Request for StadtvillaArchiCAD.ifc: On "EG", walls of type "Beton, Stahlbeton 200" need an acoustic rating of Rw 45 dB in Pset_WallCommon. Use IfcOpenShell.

First a look at what the model holds.

```python
import ifcopenshell
import ifcopenshell.util.element

model = ifcopenshell.open("StadtvillaArchiCAD.ifc")
print(model.schema)
storey = next(s for s in model.by_type("IfcBuildingStorey") if s.Name == "EG")
walls = [e for e in ifcopenshell.util.element.get_decomposition(storey) if e.is_a("IfcWall")]
seen = {}
for e in walls:
    element_type = ifcopenshell.util.element.get_type(e)
    key = (element_type.Name if element_type != e and element_type else None, ifcopenshell.util.element.get_pset(e, "Pset_WallCommon", "AcousticRating"))
    seen[key] = seen.get(key, 0) + 1
for (name, value), count in sorted(seen.items(), key=str):
    print(count, "x", name, "|", value)
```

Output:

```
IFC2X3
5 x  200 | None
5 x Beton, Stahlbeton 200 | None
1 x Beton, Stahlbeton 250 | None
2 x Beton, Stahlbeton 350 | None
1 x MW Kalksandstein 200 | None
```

```python
import ifcopenshell
import ifcopenshell.api.pset
import ifcopenshell.util.element

model = ifcopenshell.open("StadtvillaArchiCAD.ifc")

storey = next(s for s in model.by_type("IfcBuildingStorey") if s.Name == "EG")
walls = [e for e in ifcopenshell.util.element.get_decomposition(storey) if e.is_a("IfcWall")]

count = 0
for e in walls:
    element_type = ifcopenshell.util.element.get_type(e)
    if element_type in (None, e) or element_type.Name != "Beton, Stahlbeton 200":
        continue
    # add_pset returns the element's existing set when there is one.
    pset = ifcopenshell.api.pset.add_pset(model, product=e, name="Pset_WallCommon")
    ifcopenshell.api.pset.edit_pset(model, pset=pset, properties={"AcousticRating": "Rw 45 dB"})
    count += 1

print(count, "walls updated")

model.write("StadtvillaArchiCAD-out.ifc")
```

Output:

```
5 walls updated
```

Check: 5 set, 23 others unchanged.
